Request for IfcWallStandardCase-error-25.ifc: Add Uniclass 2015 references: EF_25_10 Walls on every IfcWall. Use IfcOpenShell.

First a look at what the model holds.

```python
import ifcopenshell

model = ifcopenshell.open("IfcWallStandardCase-error-25.ifc")
print(model.schema)
print("classifications:", [c.Name for c in model.by_type("IfcClassification")])
for ifc_class in ("IfcDoor", "IfcRoof", "IfcStair", "IfcWall", "IfcWindow"):
    print(ifc_class, len(model.by_type(ifc_class)))
```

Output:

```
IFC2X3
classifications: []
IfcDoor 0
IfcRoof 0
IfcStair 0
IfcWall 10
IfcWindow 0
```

```python
import ifcopenshell
import ifcopenshell.api.classification

model = ifcopenshell.open("IfcWallStandardCase-error-25.ifc")

# IFC2X3 requires Source and Edition and has no link from the project to the system.
system = model.create_entity("IfcClassification", Source="NBS", Edition="2015", Name="Uniclass 2015")

codes = {
    "IfcWall": ("EF_25_10", "Walls"),
}
for ifc_class, (code, name) in codes.items():
    products = model.by_type(ifc_class)
    ifcopenshell.api.classification.add_reference(
        model, products=products, classification=system, identification=code, name=name
    )
    print(code, len(products))

model.write("IfcWallStandardCase-error-25_v2.ifc")
```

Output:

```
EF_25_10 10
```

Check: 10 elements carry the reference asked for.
